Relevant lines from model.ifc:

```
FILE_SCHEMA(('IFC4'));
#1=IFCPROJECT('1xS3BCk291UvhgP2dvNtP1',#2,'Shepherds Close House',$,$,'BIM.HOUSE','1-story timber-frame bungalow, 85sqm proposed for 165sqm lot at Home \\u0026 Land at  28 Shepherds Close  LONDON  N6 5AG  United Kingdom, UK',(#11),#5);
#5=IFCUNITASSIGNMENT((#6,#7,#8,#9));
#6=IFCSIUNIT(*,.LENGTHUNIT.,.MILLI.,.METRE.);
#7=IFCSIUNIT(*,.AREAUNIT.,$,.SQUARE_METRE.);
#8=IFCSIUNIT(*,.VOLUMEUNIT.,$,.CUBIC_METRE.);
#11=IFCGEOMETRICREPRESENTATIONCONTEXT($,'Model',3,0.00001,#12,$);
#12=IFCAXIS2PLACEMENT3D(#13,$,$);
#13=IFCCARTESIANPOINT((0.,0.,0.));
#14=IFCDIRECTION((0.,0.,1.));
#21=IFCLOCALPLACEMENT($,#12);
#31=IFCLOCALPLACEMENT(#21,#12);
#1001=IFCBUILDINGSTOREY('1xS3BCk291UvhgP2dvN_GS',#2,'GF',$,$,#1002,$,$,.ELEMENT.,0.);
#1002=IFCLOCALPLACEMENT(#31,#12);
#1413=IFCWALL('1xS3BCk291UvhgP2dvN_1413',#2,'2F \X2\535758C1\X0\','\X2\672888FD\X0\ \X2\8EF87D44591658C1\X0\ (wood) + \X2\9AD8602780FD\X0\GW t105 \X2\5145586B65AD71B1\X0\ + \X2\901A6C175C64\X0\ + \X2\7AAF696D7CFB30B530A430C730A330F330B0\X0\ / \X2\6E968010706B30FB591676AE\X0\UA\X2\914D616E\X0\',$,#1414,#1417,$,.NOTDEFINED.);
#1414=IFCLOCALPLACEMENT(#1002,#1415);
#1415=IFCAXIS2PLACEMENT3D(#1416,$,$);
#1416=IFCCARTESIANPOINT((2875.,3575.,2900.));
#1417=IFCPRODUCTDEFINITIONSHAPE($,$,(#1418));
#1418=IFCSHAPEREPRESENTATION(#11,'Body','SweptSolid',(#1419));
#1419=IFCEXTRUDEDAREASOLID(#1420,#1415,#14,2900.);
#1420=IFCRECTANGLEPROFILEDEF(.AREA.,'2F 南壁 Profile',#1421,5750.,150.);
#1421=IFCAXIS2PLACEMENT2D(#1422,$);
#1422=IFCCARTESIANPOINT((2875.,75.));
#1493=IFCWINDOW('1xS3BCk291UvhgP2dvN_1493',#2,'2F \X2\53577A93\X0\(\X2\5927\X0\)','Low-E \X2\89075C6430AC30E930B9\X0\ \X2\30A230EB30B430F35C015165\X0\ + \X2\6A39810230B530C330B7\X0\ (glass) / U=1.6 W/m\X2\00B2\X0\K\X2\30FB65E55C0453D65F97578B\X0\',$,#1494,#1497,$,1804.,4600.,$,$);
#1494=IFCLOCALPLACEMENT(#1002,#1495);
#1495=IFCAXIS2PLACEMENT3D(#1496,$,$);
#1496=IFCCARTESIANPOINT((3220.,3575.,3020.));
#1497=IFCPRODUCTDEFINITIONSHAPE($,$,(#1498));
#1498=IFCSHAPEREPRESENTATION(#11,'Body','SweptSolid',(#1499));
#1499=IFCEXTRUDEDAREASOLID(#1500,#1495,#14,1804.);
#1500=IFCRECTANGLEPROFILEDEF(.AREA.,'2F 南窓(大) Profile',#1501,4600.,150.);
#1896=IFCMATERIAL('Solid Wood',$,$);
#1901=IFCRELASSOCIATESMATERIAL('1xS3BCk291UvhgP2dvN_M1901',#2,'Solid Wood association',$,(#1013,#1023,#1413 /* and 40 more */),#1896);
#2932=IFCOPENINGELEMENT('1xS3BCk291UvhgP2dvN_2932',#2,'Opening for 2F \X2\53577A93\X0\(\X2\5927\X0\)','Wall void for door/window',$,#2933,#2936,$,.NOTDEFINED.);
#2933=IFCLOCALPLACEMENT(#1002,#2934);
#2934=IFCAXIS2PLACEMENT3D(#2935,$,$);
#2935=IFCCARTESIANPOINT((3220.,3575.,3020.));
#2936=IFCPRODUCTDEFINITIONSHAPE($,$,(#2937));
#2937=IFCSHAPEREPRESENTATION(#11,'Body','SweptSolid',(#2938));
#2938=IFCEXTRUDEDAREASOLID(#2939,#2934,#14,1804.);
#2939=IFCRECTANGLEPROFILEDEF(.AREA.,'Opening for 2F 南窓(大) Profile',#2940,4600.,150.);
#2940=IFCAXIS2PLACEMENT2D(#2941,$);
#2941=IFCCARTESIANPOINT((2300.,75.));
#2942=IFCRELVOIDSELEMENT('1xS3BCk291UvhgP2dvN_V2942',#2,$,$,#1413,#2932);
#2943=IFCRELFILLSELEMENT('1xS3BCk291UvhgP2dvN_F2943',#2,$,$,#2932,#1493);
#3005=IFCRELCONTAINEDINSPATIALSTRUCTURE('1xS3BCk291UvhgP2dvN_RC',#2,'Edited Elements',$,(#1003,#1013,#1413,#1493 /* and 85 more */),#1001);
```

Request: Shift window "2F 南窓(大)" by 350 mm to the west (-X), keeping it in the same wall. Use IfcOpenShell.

```python
import ifcopenshell
import ifcopenshell.api.geometry
import ifcopenshell.util.placement
import ifcopenshell.util.unit

model = ifcopenshell.open("model.ifc")
unit_scale = ifcopenshell.util.unit.calculate_unit_scale(model)

window = model.by_guid("1xS3BCk291UvhgP2dvN_1493")
opening = window.FillsVoids[0].RelatingOpeningElement
wall = opening.VoidsElements[0].RelatingBuildingElement

wall_matrix = ifcopenshell.util.placement.get_local_placement(wall.ObjectPlacement)
shift = wall_matrix[:3, 0] * -0.35 / unit_scale
before = ifcopenshell.util.placement.get_local_placement(window.ObjectPlacement)[:3, 3].copy()

# The window is not placed relative to its opening, so move both.
for product in (opening, window):
    matrix = ifcopenshell.util.placement.get_local_placement(product.ObjectPlacement)
    matrix[:3, 3] += shift
    ifcopenshell.api.geometry.edit_object_placement(model, product=product, matrix=matrix, is_si=False)

after = ifcopenshell.util.placement.get_local_placement(window.ObjectPlacement)[:3, 3]
print("window moved by", (after - before).round(3) + 0.0)

model.write("model_rev.ifc")
```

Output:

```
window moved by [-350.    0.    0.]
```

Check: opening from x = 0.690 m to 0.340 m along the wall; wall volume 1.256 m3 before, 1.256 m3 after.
